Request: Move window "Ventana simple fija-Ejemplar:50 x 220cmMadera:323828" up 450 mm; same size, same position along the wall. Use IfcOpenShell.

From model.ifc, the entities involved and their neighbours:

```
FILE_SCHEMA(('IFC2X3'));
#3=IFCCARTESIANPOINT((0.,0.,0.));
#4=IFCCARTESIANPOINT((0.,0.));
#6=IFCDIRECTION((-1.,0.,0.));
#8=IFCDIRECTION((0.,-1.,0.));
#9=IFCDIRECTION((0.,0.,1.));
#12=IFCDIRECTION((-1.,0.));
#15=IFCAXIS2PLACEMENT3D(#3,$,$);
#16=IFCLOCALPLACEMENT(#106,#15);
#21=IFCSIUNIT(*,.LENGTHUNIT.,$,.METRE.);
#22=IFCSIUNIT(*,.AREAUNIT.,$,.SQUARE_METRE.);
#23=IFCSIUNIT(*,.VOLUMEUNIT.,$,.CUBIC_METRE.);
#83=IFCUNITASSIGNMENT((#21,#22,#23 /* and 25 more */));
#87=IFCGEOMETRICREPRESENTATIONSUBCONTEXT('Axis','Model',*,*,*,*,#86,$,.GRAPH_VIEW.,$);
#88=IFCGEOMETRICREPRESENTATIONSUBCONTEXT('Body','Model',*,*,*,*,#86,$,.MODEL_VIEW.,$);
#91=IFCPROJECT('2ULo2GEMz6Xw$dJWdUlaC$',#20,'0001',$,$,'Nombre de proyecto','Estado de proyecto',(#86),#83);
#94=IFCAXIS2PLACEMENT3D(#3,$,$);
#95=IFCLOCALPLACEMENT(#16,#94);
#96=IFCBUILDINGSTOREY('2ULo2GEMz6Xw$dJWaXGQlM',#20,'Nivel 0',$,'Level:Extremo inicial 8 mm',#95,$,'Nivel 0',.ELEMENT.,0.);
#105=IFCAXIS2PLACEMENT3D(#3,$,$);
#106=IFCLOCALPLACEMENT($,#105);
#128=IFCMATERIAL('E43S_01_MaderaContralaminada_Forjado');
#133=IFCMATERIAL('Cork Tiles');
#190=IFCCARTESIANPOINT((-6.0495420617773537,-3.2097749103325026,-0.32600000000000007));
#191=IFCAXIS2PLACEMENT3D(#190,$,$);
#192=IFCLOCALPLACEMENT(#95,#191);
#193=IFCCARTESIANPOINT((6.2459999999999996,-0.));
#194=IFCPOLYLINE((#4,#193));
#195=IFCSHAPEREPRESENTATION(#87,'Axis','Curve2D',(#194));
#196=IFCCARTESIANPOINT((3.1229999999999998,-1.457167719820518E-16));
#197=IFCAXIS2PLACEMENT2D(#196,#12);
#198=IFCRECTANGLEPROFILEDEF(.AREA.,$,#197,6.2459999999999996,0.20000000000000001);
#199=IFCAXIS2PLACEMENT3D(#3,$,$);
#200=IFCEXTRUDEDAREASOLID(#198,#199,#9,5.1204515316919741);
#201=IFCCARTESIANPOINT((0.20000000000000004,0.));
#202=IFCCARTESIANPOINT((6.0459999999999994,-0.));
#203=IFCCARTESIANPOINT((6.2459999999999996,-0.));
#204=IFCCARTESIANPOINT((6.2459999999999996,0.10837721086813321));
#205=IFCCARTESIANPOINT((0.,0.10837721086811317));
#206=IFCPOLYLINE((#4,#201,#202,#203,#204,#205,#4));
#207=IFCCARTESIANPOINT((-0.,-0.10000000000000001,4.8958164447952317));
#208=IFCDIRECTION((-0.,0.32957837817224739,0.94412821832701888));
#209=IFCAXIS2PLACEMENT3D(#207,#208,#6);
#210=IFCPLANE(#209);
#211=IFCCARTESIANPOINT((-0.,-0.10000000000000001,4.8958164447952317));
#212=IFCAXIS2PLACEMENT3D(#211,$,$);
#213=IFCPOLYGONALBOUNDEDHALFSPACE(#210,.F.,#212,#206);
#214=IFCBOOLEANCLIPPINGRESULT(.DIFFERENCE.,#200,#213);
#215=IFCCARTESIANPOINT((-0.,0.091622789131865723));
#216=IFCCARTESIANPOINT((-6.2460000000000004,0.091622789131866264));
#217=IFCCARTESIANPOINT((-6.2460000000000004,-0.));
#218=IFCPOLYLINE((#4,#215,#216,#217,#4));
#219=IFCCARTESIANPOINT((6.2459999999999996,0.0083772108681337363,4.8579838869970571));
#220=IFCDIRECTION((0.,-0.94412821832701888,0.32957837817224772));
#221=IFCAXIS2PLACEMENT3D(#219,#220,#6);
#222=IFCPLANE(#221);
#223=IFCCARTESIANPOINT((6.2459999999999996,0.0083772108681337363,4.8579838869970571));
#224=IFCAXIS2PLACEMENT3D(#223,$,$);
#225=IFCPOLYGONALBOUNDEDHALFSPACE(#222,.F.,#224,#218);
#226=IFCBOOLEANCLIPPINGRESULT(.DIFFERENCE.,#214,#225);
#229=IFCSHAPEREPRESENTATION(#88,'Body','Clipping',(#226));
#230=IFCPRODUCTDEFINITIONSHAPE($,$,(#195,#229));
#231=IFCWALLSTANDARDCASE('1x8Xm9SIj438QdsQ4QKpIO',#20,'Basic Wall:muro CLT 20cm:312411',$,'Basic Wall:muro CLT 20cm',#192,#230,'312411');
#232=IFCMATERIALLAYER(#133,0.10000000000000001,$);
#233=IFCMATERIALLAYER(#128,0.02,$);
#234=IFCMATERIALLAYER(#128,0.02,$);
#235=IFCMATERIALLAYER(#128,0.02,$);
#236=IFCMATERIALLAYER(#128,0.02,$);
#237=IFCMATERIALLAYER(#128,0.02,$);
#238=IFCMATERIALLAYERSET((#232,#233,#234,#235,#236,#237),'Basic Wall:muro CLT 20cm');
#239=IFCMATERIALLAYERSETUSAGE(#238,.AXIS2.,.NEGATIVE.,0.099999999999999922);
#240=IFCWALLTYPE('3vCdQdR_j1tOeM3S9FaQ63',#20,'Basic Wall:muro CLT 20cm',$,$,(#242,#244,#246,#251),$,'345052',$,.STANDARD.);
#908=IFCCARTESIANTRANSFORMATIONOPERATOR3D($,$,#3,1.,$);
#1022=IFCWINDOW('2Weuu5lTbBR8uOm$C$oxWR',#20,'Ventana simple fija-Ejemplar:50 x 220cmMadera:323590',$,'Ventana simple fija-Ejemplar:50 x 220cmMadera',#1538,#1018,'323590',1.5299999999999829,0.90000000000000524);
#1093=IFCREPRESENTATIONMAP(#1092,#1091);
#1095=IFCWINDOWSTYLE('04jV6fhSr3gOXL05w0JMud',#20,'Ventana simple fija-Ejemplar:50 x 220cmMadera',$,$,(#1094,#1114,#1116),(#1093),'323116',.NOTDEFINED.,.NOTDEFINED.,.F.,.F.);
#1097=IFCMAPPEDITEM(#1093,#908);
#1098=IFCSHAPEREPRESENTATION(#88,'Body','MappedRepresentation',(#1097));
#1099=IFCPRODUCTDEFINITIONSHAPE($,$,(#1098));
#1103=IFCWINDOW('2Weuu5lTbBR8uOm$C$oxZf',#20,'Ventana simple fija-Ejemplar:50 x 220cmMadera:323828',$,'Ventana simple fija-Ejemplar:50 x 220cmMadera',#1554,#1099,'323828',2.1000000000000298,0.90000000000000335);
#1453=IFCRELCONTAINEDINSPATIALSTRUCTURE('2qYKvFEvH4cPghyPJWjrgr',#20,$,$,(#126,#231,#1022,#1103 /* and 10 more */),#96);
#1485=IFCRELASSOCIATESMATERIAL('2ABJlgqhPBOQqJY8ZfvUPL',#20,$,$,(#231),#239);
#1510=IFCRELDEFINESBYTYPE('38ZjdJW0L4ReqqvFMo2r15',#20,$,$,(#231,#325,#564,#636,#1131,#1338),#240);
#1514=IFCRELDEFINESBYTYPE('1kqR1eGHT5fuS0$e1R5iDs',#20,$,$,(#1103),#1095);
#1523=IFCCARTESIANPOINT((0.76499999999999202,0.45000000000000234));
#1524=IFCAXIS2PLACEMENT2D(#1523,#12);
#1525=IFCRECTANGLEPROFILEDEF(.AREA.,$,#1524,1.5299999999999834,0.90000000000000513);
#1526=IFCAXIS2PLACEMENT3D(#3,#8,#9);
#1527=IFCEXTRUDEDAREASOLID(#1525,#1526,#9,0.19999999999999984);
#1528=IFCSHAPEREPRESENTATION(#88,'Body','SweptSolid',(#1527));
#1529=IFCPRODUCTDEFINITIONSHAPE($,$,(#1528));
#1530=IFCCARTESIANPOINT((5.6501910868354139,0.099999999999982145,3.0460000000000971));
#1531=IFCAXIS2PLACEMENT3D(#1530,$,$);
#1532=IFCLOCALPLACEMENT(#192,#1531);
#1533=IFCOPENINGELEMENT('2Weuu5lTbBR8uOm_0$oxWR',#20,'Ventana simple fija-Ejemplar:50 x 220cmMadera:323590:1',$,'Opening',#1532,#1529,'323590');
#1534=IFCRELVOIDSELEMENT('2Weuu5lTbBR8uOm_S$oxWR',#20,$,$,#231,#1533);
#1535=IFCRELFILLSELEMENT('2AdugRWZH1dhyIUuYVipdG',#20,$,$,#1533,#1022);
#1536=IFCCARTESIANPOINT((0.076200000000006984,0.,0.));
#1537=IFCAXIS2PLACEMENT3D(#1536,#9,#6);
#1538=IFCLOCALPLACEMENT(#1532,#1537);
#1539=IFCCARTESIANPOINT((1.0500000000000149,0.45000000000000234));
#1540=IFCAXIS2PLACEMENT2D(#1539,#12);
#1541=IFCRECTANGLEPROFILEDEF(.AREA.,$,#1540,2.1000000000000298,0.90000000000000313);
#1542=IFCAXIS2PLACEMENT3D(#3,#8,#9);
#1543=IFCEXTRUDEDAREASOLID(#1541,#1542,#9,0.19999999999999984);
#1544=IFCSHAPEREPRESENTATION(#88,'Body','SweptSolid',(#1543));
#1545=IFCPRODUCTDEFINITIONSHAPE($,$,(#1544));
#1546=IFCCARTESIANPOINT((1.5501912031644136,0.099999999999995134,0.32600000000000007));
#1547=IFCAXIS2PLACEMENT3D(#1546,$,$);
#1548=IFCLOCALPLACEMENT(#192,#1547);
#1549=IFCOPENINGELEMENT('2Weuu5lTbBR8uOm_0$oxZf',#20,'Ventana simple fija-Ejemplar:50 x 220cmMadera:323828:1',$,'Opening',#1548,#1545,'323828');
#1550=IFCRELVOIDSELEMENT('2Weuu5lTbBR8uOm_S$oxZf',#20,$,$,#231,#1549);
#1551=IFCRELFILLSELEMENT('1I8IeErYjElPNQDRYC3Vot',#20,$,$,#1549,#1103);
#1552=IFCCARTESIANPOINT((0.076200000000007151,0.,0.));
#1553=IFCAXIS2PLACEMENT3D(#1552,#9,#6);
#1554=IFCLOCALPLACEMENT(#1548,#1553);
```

```python
import numpy as np
import ifcopenshell
import ifcopenshell.api.geometry
import ifcopenshell.util.placement
import ifcopenshell.util.unit

model = ifcopenshell.open("model.ifc")
unit_scale = ifcopenshell.util.unit.calculate_unit_scale(model)

window = model.by_id(1103)
opening = window.FillsVoids[0].RelatingOpeningElement
dz = 0.45 / unit_scale

shift = np.array([0.0, 0.0, dz])
# The window is placed relative to its opening, so it follows when the opening moves.
matrix = ifcopenshell.util.placement.get_local_placement(opening.ObjectPlacement)
matrix[:3, 3] += shift
ifcopenshell.api.geometry.edit_object_placement(
    model, product=opening, matrix=matrix, is_si=False, should_transform_children=True
)

print(f"moved by {dz * unit_scale:+.3f} m")

model.write("model_rev.ifc")
```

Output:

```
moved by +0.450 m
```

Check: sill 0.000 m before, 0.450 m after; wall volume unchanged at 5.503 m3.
